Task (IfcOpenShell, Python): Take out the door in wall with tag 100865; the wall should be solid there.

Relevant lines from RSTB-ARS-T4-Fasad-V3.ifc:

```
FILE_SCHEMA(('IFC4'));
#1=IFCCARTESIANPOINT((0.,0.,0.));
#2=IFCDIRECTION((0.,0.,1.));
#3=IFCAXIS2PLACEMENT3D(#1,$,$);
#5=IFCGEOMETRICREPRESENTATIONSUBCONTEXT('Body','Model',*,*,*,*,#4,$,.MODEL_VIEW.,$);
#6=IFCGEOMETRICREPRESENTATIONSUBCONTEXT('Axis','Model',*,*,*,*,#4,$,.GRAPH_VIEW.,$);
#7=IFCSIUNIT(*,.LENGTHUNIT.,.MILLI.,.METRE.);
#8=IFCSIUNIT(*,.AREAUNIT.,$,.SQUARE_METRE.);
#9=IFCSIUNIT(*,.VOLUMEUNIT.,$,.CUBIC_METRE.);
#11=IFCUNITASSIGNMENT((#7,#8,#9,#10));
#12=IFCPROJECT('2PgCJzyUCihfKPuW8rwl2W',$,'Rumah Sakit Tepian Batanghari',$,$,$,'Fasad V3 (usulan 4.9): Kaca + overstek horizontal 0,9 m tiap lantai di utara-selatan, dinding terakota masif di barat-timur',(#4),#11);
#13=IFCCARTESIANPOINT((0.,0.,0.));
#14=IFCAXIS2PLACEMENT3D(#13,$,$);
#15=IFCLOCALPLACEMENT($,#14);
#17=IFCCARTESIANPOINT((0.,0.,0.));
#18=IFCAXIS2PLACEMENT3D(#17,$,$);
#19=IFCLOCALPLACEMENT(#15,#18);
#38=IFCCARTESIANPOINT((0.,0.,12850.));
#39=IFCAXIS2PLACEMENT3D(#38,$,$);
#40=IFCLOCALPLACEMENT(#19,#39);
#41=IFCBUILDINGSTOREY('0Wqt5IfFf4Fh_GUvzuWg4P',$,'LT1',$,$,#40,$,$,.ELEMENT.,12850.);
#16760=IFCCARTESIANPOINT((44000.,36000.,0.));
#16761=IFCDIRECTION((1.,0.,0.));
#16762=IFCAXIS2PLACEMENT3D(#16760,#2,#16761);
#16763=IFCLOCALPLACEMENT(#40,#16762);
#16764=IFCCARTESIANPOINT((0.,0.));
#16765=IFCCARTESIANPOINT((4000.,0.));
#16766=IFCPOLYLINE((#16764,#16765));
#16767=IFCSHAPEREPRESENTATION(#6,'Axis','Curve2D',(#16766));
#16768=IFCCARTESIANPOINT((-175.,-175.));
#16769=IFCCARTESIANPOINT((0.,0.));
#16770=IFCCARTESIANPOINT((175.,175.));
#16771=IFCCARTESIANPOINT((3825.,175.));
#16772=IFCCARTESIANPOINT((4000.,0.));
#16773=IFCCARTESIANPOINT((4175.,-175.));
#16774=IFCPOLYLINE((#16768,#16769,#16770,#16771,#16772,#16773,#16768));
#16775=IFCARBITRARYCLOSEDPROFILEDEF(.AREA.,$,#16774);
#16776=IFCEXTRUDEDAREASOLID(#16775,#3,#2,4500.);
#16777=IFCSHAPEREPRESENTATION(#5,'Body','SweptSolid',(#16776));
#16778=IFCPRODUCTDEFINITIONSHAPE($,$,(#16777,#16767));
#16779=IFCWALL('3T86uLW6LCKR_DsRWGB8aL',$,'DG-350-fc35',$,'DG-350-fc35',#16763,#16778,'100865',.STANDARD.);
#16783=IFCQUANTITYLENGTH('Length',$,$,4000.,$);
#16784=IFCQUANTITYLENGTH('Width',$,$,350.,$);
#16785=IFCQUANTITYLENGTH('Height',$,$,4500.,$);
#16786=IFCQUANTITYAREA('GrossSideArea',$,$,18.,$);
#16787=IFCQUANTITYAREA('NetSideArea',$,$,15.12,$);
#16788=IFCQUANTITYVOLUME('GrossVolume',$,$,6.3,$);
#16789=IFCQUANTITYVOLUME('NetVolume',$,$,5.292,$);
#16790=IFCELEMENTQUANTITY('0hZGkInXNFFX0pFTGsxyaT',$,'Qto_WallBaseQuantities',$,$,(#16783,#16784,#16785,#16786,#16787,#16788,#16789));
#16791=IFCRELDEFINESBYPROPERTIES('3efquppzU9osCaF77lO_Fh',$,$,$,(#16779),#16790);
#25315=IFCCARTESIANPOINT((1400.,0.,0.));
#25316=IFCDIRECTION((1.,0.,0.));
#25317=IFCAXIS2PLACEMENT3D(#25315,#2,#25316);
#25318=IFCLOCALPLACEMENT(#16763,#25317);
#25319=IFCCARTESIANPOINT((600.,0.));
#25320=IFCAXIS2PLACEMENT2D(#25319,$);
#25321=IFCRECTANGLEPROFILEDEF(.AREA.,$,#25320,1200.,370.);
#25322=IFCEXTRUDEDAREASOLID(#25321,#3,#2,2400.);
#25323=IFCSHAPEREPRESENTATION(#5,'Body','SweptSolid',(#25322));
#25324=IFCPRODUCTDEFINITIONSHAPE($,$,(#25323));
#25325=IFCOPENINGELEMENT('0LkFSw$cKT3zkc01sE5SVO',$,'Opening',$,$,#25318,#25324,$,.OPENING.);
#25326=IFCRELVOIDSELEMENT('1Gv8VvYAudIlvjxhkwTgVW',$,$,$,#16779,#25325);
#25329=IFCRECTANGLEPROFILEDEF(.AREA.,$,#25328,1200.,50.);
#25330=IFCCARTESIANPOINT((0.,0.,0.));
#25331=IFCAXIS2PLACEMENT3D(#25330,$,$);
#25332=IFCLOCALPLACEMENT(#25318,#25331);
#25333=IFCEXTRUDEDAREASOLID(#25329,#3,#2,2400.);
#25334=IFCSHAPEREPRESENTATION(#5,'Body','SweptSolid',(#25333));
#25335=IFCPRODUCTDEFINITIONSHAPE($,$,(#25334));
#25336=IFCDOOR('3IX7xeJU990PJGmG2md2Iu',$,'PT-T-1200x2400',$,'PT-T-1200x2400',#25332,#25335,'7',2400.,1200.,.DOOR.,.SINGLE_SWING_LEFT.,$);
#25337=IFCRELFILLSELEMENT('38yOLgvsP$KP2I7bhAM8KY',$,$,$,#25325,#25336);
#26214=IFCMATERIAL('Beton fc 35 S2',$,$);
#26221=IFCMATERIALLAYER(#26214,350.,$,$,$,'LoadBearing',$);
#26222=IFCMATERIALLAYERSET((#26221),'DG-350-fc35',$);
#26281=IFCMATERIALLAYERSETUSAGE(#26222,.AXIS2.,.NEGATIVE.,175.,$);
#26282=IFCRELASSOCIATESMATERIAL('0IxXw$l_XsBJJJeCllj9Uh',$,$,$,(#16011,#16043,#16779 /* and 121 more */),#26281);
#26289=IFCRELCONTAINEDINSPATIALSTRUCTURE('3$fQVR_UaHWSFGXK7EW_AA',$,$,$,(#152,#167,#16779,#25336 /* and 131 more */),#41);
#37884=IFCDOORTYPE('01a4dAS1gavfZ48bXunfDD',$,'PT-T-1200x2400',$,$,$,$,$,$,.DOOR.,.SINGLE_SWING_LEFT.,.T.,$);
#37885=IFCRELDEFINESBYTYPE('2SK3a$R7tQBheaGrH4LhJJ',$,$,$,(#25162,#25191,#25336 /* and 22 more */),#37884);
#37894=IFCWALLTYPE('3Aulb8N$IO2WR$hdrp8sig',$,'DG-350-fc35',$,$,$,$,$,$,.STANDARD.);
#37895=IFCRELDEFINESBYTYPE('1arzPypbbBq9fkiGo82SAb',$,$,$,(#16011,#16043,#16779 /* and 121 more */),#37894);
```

```python
import ifcopenshell
import ifcopenshell.api.feature
import ifcopenshell.api.pset
import ifcopenshell.api.root
import ifcopenshell.geom
import ifcopenshell.util.element
import ifcopenshell.util.shape
import ifcopenshell.util.unit

model = ifcopenshell.open("RSTB-ARS-T4-Fasad-V3.ifc")
area_scale = ifcopenshell.util.unit.calculate_unit_scale(model, "AREAUNIT")
volume_scale = ifcopenshell.util.unit.calculate_unit_scale(model, "VOLUMEUNIT")
settings = ifcopenshell.geom.settings()


def volume(element):
    """Net volume in cubic metres, openings subtracted."""
    shape = ifcopenshell.geom.create_shape(settings, element)
    return ifcopenshell.util.shape.get_volume(shape.geometry)


door = model.by_guid("3IX7xeJU990PJGmG2md2Iu")
opening = door.FillsVoids[0].RelatingOpeningElement
wall = opening.VoidsElements[0].RelatingBuildingElement
before = volume(wall)

ifcopenshell.api.root.remove_product(model, product=door)
ifcopenshell.api.feature.remove_feature(model, feature=opening)

after = volume(wall)
thickness = 0.35  # wall thickness in metres

# Update the wall's stored quantities.
qto = model.by_id(ifcopenshell.util.element.get_pset(wall, "Qto_WallBaseQuantities", should_inherit=False)["id"])
ifcopenshell.api.pset.edit_qto(model, qto=qto, properties={
    "NetSideArea": after / thickness / area_scale,
    "NetVolume": after / volume_scale,
})

print(f"wall volume {before:.3f} -> {after:.3f} m3")

model.write("RSTB-ARS-T4-Fasad-V3_v2.ifc")
```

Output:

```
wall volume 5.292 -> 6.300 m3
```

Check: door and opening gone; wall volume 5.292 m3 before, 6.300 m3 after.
